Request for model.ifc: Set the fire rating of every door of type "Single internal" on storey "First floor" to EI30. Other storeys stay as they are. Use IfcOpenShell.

First a look at what the model holds.

```python
import ifcopenshell
import ifcopenshell.util.element

model = ifcopenshell.open("model.ifc")
print(model.schema)
storey = next(s for s in model.by_type("IfcBuildingStorey") if s.Name == "First floor")
doors = [e for e in ifcopenshell.util.element.get_decomposition(storey) if e.is_a("IfcDoor")]
seen = {}
for e in doors:
    element_type = ifcopenshell.util.element.get_type(e)
    key = (element_type.Name if element_type != e and element_type else None, ifcopenshell.util.element.get_pset(e, "Pset_DoorCommon", "FireRating"))
    seen[key] = seen.get(key, 0) + 1
for (name, value), count in sorted(seen.items(), key=str):
    print(count, "x", name, "|", value)
```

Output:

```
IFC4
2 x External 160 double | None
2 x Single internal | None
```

```python
import ifcopenshell
import ifcopenshell.api.pset
import ifcopenshell.util.element

model = ifcopenshell.open("model.ifc")

storey = next(s for s in model.by_type("IfcBuildingStorey") if s.Name == "First floor")
doors = [e for e in ifcopenshell.util.element.get_decomposition(storey) if e.is_a("IfcDoor")]

count = 0
for e in doors:
    element_type = ifcopenshell.util.element.get_type(e)
    if element_type in (None, e) or element_type.Name != "Single internal":
        continue
    # add_pset returns the element's existing set when there is one.
    pset = ifcopenshell.api.pset.add_pset(model, product=e, name="Pset_DoorCommon")
    ifcopenshell.api.pset.edit_pset(model, pset=pset, properties={"FireRating": "EI30"})
    count += 1

print(count, "doors updated")

model.write("model_updated.ifc")
```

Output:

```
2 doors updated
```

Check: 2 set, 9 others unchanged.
